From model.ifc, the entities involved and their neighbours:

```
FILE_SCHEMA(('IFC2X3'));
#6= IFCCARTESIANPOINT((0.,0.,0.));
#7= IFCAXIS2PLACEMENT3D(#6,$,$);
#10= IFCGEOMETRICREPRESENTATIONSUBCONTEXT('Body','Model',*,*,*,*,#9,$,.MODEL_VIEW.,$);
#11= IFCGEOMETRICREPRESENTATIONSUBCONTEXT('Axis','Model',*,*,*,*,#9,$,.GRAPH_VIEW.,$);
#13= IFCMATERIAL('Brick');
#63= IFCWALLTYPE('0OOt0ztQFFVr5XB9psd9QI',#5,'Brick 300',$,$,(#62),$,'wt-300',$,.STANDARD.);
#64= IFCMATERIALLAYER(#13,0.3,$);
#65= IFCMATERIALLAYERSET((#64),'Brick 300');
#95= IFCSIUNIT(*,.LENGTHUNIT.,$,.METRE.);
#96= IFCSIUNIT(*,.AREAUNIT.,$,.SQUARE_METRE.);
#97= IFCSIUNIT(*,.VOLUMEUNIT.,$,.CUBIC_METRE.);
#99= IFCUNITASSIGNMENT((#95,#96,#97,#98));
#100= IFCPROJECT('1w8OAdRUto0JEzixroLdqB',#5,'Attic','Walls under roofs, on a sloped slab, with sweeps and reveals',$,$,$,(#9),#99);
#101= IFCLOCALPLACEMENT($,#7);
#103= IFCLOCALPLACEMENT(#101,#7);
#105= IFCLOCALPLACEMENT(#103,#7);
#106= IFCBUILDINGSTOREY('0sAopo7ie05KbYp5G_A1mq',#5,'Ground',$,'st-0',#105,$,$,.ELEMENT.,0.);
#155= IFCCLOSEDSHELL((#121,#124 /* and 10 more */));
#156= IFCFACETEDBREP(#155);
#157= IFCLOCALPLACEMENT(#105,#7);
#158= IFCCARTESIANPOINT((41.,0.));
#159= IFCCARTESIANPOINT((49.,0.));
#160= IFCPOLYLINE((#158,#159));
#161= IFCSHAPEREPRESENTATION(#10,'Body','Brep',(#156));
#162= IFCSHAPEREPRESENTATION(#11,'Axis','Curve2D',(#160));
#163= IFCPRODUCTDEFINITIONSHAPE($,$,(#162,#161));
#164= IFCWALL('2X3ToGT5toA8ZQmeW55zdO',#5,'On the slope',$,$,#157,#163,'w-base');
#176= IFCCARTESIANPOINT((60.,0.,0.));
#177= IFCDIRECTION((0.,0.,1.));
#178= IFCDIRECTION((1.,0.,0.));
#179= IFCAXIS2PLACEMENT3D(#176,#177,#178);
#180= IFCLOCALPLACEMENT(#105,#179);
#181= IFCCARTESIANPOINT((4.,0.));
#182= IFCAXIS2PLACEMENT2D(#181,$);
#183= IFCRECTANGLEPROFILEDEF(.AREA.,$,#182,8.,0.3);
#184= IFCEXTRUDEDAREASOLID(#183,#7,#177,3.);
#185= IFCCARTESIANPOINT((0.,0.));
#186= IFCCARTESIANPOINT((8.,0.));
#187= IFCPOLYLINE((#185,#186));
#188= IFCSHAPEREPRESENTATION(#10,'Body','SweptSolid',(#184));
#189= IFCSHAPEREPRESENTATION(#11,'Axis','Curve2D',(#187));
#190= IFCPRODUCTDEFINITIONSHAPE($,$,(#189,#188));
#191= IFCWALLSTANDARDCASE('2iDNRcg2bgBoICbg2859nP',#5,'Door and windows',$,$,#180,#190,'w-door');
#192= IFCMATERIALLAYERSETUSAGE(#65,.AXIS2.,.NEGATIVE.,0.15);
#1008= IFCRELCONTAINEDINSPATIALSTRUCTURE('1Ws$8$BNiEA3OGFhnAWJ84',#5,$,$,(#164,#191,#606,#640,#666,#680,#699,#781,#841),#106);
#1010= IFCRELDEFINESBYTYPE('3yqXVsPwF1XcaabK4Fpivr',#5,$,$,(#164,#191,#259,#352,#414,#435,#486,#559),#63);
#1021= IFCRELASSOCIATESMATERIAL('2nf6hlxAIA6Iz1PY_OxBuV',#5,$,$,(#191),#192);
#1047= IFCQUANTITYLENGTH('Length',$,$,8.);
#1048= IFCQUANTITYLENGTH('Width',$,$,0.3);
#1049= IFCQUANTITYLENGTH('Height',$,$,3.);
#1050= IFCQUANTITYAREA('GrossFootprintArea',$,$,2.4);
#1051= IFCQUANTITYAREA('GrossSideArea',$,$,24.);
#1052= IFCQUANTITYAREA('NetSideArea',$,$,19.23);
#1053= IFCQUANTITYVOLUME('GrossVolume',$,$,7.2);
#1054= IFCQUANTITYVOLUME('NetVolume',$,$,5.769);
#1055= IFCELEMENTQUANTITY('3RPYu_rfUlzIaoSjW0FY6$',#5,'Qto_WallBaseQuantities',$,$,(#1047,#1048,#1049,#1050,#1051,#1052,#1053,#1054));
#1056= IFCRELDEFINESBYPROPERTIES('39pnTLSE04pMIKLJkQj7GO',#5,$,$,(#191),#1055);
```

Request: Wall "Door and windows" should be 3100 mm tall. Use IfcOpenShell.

```python
import ifcopenshell
import ifcopenshell.api.pset
import ifcopenshell.geom
import ifcopenshell.util.element
import ifcopenshell.util.representation
import ifcopenshell.util.shape
import ifcopenshell.util.unit

model = ifcopenshell.open("model.ifc")
unit_scale = ifcopenshell.util.unit.calculate_unit_scale(model)
area_scale = ifcopenshell.util.unit.calculate_unit_scale(model, "AREAUNIT")
volume_scale = ifcopenshell.util.unit.calculate_unit_scale(model, "VOLUMEUNIT")
settings = ifcopenshell.geom.settings()


def volume(element):
    """Net volume in cubic metres, openings subtracted."""
    shape = ifcopenshell.geom.create_shape(settings, element)
    return ifcopenshell.util.shape.get_volume(shape.geometry)


wall = model.by_guid("2iDNRcg2bgBoICbg2859nP")
before = volume(wall)

body = ifcopenshell.util.representation.get_representation(wall, "Model", "Body")
solid = body.Items[0]
old_height = solid.Depth
solid.Depth = 3.1 / unit_scale
after = volume(wall)
thickness = 0.3  # wall thickness in metres

# Update the stored height, areas and volumes.
qto = model.by_id(ifcopenshell.util.element.get_pset(wall, "Qto_WallBaseQuantities", should_inherit=False)["id"])
ifcopenshell.api.pset.edit_qto(model, qto=qto, properties={
    "Height": solid.Depth,
    "GrossSideArea": ifcopenshell.util.element.get_pset(wall, "Qto_WallBaseQuantities", "GrossSideArea") * solid.Depth / old_height,
    "NetSideArea": after / thickness / area_scale,
    "GrossVolume": ifcopenshell.util.element.get_pset(wall, "Qto_WallBaseQuantities", "GrossVolume") * solid.Depth / old_height,
    "NetVolume": after / volume_scale,
})

print(f"height {old_height:g} -> {solid.Depth:g}, volume {before:.3f} -> {after:.3f} m3")

model.write("model_edited.ifc")
```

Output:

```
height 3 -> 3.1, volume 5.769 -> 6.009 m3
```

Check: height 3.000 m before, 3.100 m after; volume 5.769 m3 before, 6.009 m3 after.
